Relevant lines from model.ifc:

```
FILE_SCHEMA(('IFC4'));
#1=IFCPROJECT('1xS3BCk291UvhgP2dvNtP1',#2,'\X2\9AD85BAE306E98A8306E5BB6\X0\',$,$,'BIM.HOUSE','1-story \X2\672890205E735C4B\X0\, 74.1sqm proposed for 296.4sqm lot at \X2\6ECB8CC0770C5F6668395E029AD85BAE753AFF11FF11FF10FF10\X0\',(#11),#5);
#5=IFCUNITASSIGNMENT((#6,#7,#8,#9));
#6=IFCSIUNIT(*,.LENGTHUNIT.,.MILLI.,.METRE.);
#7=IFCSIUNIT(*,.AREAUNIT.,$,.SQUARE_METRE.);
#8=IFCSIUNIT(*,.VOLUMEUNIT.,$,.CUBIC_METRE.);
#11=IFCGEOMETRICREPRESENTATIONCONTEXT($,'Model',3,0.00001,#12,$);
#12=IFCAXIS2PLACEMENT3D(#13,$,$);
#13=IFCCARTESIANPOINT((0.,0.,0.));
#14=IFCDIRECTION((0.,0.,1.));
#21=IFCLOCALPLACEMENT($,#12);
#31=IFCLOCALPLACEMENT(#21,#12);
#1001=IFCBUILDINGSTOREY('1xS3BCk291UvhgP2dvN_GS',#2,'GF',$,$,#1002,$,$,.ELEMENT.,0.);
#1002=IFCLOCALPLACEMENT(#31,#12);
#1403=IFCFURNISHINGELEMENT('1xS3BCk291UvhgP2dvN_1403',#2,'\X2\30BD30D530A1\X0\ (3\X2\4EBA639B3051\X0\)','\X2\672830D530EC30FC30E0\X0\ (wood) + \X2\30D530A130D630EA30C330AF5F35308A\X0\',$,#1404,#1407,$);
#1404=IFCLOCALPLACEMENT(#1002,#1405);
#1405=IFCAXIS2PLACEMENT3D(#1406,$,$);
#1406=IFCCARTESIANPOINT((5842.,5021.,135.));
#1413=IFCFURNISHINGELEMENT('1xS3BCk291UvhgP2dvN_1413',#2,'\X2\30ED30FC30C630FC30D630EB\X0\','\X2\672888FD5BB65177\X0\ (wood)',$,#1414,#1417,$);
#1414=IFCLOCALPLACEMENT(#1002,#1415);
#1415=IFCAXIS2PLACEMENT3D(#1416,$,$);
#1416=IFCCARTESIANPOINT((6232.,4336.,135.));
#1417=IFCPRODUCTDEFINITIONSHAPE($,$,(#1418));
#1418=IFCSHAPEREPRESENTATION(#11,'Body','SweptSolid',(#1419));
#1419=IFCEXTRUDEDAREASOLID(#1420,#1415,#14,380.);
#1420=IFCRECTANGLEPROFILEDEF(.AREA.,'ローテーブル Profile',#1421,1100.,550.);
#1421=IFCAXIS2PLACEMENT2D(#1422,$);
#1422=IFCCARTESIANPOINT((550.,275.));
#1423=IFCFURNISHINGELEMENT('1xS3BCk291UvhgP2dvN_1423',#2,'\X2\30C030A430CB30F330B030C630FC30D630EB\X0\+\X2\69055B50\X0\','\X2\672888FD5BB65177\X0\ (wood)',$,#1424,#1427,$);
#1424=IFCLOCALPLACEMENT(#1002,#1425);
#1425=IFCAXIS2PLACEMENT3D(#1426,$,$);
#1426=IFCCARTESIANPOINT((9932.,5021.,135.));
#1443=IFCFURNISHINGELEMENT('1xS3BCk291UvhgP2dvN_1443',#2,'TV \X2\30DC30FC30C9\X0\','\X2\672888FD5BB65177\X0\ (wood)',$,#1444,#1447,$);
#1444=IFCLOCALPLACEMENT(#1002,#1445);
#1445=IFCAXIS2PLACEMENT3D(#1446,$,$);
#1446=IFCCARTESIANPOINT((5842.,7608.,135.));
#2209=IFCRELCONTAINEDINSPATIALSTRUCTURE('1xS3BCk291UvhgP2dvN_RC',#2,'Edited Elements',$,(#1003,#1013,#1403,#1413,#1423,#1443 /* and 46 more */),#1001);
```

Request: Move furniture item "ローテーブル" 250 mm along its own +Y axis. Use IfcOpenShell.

```python
import ifcopenshell
import ifcopenshell.api.geometry
import ifcopenshell.util.placement
import ifcopenshell.util.unit

model = ifcopenshell.open("model.ifc")
unit_scale = ifcopenshell.util.unit.calculate_unit_scale(model)

item = model.by_id(1413)
matrix = ifcopenshell.util.placement.get_local_placement(item.ObjectPlacement)
matrix[:3, 3] += matrix[:3, 1] * 0.25 / unit_scale
ifcopenshell.api.geometry.edit_object_placement(model, product=item, matrix=matrix, is_si=False)

print(ifcopenshell.util.placement.get_local_placement(item.ObjectPlacement).round(3) + 0.0)

model.write("model_edited.ifc")
```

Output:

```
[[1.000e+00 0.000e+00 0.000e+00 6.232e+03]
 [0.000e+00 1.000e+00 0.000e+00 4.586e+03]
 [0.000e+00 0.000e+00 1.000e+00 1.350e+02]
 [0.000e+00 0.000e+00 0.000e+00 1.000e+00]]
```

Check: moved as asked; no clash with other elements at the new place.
